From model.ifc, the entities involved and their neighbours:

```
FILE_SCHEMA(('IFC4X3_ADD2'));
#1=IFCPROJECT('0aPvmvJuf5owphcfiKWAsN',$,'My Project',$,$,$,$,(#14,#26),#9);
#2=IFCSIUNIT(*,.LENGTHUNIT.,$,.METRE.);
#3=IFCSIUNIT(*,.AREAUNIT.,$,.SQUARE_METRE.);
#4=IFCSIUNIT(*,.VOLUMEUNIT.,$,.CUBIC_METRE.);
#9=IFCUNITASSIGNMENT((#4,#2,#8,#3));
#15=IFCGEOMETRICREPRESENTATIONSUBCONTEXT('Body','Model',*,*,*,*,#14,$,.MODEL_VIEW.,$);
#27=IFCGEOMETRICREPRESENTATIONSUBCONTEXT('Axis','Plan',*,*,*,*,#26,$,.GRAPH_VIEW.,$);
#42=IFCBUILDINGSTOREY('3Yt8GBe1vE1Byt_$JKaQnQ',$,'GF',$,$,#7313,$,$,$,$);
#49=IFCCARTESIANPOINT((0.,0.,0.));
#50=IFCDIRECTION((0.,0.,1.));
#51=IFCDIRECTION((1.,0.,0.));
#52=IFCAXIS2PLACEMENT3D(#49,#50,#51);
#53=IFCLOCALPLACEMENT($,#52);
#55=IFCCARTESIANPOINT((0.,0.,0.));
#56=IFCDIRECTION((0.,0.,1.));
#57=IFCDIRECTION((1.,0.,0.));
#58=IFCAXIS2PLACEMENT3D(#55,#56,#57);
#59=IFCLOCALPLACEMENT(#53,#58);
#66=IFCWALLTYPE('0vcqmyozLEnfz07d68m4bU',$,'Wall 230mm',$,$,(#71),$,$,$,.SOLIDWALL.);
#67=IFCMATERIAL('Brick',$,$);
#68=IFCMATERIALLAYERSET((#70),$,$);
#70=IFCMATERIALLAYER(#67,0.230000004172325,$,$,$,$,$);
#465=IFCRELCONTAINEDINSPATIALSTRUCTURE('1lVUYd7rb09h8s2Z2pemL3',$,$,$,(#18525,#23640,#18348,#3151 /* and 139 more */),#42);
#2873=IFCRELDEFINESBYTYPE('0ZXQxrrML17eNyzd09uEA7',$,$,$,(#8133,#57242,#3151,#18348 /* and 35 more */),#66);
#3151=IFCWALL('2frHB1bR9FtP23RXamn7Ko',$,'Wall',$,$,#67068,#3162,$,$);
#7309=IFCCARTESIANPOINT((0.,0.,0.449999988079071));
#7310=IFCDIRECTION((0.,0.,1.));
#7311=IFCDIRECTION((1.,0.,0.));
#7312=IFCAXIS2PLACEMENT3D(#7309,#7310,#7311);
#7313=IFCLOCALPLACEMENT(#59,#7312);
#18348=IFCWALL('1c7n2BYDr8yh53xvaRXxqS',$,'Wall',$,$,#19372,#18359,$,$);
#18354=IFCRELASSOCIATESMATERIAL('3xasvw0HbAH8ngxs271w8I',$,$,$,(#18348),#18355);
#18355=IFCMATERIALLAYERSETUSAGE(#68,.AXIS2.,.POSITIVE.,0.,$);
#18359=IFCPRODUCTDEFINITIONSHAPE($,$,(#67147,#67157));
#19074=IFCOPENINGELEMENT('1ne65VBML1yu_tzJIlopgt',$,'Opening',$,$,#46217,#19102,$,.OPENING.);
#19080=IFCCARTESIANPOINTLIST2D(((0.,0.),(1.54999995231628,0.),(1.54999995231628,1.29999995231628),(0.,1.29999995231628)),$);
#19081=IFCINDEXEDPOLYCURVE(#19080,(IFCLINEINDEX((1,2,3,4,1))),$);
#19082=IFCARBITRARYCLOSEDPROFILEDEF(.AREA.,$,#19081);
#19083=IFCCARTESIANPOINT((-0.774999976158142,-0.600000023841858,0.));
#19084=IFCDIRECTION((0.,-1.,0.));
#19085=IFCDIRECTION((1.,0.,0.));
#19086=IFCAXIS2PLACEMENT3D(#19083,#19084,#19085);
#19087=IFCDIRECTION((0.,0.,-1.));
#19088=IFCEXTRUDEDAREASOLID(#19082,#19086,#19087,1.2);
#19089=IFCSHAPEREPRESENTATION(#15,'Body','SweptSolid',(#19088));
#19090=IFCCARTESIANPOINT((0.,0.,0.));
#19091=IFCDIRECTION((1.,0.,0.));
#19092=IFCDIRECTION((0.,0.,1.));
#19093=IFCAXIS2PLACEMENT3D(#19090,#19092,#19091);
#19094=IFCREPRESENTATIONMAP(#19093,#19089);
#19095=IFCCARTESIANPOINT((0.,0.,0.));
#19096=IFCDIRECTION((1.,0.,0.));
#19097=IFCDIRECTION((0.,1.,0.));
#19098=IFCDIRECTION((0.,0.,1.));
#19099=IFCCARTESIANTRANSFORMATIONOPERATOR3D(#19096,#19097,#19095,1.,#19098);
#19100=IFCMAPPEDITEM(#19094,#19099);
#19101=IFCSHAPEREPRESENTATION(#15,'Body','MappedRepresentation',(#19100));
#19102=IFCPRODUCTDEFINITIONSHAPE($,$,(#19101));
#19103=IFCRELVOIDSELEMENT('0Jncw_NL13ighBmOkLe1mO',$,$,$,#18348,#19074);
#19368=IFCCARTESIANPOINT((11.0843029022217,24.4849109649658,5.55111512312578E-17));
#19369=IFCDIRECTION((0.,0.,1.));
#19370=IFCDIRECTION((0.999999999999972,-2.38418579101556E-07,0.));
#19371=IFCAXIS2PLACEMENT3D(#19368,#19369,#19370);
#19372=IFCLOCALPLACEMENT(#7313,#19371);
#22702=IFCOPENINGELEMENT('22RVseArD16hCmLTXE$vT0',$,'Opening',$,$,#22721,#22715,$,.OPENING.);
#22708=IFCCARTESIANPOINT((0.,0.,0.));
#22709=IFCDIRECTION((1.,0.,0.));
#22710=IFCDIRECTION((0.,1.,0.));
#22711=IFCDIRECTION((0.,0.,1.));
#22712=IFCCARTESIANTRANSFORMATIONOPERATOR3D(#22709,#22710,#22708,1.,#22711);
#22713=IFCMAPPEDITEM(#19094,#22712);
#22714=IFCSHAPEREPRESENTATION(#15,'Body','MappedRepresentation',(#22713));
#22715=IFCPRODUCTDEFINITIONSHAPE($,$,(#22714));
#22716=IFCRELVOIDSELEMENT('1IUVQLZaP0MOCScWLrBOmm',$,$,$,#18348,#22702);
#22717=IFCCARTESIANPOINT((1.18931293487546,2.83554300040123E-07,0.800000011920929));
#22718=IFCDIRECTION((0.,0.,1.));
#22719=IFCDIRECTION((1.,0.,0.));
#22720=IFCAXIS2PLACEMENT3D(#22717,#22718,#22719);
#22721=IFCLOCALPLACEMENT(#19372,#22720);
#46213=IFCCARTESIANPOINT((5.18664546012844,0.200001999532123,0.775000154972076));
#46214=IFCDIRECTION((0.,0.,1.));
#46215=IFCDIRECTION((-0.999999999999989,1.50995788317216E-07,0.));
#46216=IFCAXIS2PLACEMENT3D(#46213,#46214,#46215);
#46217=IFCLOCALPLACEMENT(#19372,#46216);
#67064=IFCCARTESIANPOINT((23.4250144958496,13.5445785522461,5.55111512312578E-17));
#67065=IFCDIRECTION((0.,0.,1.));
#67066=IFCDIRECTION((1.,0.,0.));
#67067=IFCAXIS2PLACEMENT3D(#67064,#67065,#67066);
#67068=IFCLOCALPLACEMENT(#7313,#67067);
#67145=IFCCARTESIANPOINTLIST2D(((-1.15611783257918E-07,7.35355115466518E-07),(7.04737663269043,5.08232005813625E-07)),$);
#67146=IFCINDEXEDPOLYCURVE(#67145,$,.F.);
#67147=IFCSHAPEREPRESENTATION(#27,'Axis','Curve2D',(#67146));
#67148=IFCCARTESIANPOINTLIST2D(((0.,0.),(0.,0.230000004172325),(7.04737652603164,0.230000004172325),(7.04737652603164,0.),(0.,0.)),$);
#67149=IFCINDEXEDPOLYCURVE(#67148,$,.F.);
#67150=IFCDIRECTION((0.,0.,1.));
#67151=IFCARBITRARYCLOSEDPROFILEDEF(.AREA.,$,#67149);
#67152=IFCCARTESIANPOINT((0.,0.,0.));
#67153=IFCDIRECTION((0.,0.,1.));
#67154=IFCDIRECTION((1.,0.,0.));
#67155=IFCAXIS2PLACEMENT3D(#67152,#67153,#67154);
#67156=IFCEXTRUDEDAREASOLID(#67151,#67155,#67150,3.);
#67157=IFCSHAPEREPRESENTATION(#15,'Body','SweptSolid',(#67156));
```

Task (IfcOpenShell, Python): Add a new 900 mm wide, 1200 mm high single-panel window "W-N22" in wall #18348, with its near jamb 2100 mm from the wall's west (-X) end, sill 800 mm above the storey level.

```python
import numpy as np
import ifcopenshell
import ifcopenshell.api.feature
import ifcopenshell.api.geometry
import ifcopenshell.api.root
import ifcopenshell.api.spatial
import ifcopenshell.geom
import ifcopenshell.util.element
import ifcopenshell.util.placement
import ifcopenshell.util.representation
import ifcopenshell.util.shape
import ifcopenshell.util.unit

model = ifcopenshell.open("model.ifc")
unit_scale = ifcopenshell.util.unit.calculate_unit_scale(model)
settings = ifcopenshell.geom.settings()


def volume(element):
    """Net volume in cubic metres, openings subtracted."""
    shape = ifcopenshell.geom.create_shape(settings, element)
    return ifcopenshell.util.shape.get_volume(shape.geometry)


wall = model.by_guid("1c7n2BYDr8yh53xvaRXxqS")
storey = ifcopenshell.util.element.get_container(wall, ifc_class="IfcBuildingStorey")
context = ifcopenshell.util.representation.get_context(model, "Model", "Body", "MODEL_VIEW")
before = volume(wall)

width, height, from_end, sill = 0.9, 1.2, 2.1, 0.8  # metres

# The wall runs along its own X axis, and the end named is its -X end.
wall_shape = ifcopenshell.geom.create_shape(settings, wall)
x, y, z = ifcopenshell.util.shape.get_vertices(wall_shape.geometry).T
start = x.min() + from_end
face, thickness = float(y.min()), float(y.max() - y.min())
wall_matrix = ifcopenshell.util.placement.get_local_placement(wall.ObjectPlacement)
level = ifcopenshell.util.placement.get_local_placement(storey.ObjectPlacement)[2, 3]


def in_wall(x, y):
    """Placement at x, y metres in the wall's axes, at sill height."""
    matrix = wall_matrix.copy()
    matrix[:, 3] = wall_matrix @ np.array([x / unit_scale, y / unit_scale, 0.0, 1.0])
    matrix[2, 3] = level + sill / unit_scale
    return matrix


# Opening: a box that overshoots both wall faces by 50 mm.
opening = ifcopenshell.api.root.create_entity(model, ifc_class="IfcOpeningElement", predefined_type="OPENING")
box = ifcopenshell.api.geometry.add_wall_representation(
    model, context=context, length=width, height=height, thickness=thickness + 0.1
)
ifcopenshell.api.geometry.assign_representation(model, product=opening, representation=box)
ifcopenshell.api.geometry.edit_object_placement(model, product=opening, matrix=in_wall(start, face - 0.05), is_si=False)
ifcopenshell.api.feature.add_feature(model, feature=opening, element=wall)

window = ifcopenshell.api.root.create_entity(model, ifc_class="IfcWindow", name="W-N22", predefined_type="WINDOW")
window.OverallWidth, window.OverallHeight = width / unit_scale, height / unit_scale
window.PartitioningType = "SINGLE_PANEL"
body = ifcopenshell.api.geometry.add_window_representation(
    model,
    context=context,
    overall_width=window.OverallWidth,
    overall_height=window.OverallHeight,
    partition_type="SINGLE_PANEL",
)
ifcopenshell.api.geometry.assign_representation(model, product=window, representation=body)
ifcopenshell.api.spatial.assign_container(model, products=[window], relating_structure=storey)
ifcopenshell.api.feature.add_filling(model, opening=opening, element=window)

# Centre the window in the wall's thickness.
ifcopenshell.api.geometry.edit_object_placement(model, product=window, matrix=in_wall(start, face), is_si=False)
window_shape = ifcopenshell.geom.create_shape(settings, window)
depth = ifcopenshell.util.shape.get_vertices(window_shape.geometry)[:, 1]
offset = face + thickness / 2 - (depth.min() + depth.max()) / 2
ifcopenshell.api.geometry.edit_object_placement(model, product=window, matrix=in_wall(start, offset), is_si=False)

after = volume(wall)

print(f"wall volume {before:.3f} -> {after:.3f} m3")

model.write("model_updated.ifc")
```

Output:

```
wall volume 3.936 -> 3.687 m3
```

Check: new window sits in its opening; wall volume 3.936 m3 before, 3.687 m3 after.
